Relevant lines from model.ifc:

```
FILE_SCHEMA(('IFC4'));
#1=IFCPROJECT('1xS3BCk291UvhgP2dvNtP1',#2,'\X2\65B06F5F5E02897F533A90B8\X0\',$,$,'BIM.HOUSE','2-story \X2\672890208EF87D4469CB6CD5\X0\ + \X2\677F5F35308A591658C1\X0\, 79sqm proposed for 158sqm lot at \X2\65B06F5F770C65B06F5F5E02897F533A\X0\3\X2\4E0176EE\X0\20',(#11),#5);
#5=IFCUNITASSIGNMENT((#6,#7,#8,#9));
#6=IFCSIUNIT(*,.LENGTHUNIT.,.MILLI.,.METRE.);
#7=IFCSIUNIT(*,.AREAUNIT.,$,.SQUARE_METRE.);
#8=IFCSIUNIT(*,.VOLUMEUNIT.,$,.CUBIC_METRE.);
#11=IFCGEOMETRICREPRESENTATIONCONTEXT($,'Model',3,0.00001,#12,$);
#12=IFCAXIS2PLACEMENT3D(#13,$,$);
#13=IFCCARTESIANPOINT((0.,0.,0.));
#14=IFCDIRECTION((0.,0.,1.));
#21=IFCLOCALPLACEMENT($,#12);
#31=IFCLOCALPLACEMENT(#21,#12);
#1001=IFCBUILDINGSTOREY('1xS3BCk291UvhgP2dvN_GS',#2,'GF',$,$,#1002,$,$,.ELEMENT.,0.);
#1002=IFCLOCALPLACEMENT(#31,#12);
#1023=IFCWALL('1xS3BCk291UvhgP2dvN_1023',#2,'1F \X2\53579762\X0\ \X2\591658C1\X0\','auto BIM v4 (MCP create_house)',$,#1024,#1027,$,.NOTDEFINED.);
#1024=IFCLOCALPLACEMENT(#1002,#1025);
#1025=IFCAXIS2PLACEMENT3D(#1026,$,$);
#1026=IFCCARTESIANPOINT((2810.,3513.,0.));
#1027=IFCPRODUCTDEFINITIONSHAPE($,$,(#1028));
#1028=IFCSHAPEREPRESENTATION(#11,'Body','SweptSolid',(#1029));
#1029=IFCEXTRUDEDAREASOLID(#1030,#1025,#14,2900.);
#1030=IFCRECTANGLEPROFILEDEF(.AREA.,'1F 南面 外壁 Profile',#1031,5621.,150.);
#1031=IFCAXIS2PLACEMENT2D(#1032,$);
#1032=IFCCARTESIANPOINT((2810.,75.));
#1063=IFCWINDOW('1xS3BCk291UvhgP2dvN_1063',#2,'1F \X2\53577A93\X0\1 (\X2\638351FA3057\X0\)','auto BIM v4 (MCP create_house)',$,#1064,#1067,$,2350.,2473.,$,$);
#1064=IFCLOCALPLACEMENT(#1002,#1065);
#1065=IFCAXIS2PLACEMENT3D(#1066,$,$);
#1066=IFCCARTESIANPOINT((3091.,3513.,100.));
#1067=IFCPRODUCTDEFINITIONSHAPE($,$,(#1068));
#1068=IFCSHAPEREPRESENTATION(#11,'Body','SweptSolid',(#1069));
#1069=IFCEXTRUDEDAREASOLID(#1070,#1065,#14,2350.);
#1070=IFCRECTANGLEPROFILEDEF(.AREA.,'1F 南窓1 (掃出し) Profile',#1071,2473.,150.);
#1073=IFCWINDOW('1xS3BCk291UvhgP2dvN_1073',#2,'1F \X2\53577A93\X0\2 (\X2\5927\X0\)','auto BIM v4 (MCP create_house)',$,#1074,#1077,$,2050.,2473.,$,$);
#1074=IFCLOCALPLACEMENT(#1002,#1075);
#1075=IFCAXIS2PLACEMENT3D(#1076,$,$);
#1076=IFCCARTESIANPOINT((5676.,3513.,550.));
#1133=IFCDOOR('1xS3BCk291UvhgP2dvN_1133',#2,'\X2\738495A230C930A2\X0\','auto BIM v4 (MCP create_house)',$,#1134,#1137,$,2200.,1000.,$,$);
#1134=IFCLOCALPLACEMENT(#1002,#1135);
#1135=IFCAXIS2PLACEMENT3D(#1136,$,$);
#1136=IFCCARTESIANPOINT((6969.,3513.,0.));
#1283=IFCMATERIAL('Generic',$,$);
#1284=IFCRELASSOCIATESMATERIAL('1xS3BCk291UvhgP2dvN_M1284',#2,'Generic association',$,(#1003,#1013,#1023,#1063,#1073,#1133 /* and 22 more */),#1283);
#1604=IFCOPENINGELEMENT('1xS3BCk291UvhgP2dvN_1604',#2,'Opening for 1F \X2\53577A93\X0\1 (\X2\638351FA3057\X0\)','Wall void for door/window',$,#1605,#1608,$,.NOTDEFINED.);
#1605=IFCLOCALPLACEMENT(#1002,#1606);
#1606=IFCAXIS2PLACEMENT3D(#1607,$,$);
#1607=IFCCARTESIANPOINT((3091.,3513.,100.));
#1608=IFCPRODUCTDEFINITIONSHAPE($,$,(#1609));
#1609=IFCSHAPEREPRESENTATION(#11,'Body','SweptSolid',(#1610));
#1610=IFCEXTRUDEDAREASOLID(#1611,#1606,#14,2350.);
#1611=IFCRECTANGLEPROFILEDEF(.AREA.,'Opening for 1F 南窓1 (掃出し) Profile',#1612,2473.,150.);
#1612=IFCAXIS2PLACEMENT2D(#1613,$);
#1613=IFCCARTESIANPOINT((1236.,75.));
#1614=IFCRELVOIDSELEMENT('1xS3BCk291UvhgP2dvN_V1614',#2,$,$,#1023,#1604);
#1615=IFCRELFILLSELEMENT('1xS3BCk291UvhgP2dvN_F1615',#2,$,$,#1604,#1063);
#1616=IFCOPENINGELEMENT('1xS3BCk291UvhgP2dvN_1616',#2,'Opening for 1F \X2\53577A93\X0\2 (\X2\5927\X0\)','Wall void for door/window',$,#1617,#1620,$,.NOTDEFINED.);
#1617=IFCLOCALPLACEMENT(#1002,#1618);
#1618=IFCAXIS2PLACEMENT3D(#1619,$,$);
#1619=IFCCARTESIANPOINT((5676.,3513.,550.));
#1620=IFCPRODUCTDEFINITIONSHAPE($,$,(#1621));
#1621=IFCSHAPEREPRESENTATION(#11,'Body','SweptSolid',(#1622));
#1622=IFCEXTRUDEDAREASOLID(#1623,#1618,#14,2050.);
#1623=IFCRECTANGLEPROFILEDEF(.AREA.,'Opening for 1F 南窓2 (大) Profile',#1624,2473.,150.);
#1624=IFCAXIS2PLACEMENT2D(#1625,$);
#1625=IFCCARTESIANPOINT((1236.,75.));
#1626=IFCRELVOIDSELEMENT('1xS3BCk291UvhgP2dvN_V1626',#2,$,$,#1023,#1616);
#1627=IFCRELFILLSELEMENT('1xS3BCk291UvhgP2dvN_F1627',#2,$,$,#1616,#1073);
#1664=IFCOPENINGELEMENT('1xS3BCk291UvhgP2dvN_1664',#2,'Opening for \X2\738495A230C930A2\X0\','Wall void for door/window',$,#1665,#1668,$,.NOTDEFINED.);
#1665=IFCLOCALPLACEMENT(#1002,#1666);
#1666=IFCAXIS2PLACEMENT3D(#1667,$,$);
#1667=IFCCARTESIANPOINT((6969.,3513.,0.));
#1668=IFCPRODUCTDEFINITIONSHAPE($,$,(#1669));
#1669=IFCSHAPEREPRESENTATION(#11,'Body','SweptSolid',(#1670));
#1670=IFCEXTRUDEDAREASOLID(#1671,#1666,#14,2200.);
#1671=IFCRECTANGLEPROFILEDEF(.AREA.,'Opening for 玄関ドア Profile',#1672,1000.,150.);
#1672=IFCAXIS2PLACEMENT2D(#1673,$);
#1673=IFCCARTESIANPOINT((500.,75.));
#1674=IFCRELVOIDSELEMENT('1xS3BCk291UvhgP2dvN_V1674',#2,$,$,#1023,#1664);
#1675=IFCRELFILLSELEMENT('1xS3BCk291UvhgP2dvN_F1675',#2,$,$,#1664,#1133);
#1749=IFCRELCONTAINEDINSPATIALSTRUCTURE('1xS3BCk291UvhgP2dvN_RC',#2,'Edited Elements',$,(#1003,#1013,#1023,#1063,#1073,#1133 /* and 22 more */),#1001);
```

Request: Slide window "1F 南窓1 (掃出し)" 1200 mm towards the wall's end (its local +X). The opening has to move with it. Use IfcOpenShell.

```python
import ifcopenshell
import ifcopenshell.api.geometry
import ifcopenshell.util.placement
import ifcopenshell.util.unit

model = ifcopenshell.open("model.ifc")
unit_scale = ifcopenshell.util.unit.calculate_unit_scale(model)

window = model.by_guid("1xS3BCk291UvhgP2dvN_1063")
opening = window.FillsVoids[0].RelatingOpeningElement
wall = opening.VoidsElements[0].RelatingBuildingElement

wall_matrix = ifcopenshell.util.placement.get_local_placement(wall.ObjectPlacement)
shift = wall_matrix[:3, 0] * 1.2 / unit_scale
before = ifcopenshell.util.placement.get_local_placement(window.ObjectPlacement)[:3, 3].copy()

# The window is not placed relative to its opening, so move both.
for product in (opening, window):
    matrix = ifcopenshell.util.placement.get_local_placement(product.ObjectPlacement)
    matrix[:3, 3] += shift
    ifcopenshell.api.geometry.edit_object_placement(model, product=product, matrix=matrix, is_si=False)

after = ifcopenshell.util.placement.get_local_placement(window.ObjectPlacement)[:3, 3]
print("window moved by", (after - before).round(3) + 0.0)

model.write("model_updated.ifc")
```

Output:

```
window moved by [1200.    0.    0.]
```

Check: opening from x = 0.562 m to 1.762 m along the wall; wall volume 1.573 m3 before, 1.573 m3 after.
